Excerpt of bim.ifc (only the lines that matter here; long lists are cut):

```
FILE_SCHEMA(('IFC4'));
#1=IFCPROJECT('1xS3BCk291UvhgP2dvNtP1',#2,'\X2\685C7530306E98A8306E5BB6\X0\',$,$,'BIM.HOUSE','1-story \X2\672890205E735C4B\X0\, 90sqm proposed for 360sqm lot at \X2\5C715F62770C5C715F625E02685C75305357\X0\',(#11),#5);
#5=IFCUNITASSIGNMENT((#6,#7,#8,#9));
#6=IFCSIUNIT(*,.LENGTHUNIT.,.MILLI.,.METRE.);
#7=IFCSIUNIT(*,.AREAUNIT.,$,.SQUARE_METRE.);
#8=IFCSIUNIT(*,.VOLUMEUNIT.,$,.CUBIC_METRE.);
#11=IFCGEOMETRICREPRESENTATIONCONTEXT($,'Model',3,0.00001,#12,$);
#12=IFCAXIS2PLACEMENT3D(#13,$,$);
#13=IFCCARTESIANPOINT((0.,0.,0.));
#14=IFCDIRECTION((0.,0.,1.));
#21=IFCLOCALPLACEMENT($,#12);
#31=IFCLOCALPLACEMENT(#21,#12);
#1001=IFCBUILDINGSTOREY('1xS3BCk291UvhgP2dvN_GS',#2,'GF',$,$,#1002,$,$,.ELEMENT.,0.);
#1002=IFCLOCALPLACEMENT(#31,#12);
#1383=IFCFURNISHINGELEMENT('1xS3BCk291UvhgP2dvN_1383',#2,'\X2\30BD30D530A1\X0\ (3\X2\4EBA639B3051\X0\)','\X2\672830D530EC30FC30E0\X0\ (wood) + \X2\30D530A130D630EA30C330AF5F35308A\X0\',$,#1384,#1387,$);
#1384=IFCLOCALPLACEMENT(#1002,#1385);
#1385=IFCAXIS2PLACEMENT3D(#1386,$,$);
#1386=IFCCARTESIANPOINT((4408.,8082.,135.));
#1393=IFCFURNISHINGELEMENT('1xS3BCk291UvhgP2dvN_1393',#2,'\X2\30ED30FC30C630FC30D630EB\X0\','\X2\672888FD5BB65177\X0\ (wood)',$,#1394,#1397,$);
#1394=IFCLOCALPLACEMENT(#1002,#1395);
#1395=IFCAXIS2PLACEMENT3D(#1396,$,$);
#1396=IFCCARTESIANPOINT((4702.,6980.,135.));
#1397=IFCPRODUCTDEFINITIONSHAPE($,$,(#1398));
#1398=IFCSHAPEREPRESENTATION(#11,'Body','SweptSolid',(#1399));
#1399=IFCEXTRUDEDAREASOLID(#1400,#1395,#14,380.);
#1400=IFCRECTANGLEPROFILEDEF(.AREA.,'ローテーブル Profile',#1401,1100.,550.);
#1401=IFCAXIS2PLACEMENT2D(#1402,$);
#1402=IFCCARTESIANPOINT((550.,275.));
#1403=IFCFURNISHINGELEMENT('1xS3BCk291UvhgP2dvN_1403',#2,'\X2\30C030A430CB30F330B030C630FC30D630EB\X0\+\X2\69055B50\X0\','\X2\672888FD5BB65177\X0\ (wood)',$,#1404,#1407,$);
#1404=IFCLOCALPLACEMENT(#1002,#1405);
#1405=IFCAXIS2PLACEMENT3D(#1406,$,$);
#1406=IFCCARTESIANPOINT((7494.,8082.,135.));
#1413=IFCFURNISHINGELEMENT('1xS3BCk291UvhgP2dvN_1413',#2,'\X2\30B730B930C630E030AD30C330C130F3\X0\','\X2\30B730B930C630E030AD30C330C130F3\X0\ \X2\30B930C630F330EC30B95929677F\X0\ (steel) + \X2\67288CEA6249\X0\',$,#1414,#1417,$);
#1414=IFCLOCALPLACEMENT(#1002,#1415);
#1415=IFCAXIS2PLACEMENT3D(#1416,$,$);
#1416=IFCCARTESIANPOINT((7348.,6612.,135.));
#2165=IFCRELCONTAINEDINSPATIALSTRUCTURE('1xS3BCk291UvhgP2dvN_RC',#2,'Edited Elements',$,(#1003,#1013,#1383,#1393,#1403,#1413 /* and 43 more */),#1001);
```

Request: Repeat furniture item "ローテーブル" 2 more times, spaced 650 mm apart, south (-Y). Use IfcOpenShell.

```python
import numpy as np
import ifcopenshell
import ifcopenshell.api.geometry
import ifcopenshell.api.root
import ifcopenshell.util.element
import ifcopenshell.util.placement
import ifcopenshell.util.unit

model = ifcopenshell.open("bim.ifc")
unit_scale = ifcopenshell.util.unit.calculate_unit_scale(model)


def reuse_history(source, copy):
    """copy_class also copies each property set's owner history, people and application; keep the originals."""
    for rel in copy.IsDefinedBy:
        if rel.is_a("IfcRelDefinesByProperties") and (history := rel.RelatingPropertyDefinition.OwnerHistory):
            rel.RelatingPropertyDefinition.OwnerHistory = source.OwnerHistory
            ifcopenshell.util.element.remove_deep2(model, history)


source = model.by_guid("1xS3BCk291UvhgP2dvN_1393")
base = ifcopenshell.util.placement.get_local_placement(source.ObjectPlacement)
step = np.array([0.0, -1.0, 0.0]) * 0.65 / unit_scale

for i in range(1, 3):
    copy = ifcopenshell.api.root.copy_class(model, product=source)
    copy.Representation = ifcopenshell.util.element.copy_deep(
        model, source.Representation, exclude=["IfcGeometricRepresentationContext", "IfcRepresentationMap"]
    )
    reuse_history(source, copy)
    matrix = base.copy()
    matrix[:3, 3] += i * step
    print("added at", matrix[:3, 3].round(3) + 0.0)
    ifcopenshell.api.geometry.edit_object_placement(model, product=copy, matrix=matrix, is_si=False)

model.write("bim-out.ifc")
```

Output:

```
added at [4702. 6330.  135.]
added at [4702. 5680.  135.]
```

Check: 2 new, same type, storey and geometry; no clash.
